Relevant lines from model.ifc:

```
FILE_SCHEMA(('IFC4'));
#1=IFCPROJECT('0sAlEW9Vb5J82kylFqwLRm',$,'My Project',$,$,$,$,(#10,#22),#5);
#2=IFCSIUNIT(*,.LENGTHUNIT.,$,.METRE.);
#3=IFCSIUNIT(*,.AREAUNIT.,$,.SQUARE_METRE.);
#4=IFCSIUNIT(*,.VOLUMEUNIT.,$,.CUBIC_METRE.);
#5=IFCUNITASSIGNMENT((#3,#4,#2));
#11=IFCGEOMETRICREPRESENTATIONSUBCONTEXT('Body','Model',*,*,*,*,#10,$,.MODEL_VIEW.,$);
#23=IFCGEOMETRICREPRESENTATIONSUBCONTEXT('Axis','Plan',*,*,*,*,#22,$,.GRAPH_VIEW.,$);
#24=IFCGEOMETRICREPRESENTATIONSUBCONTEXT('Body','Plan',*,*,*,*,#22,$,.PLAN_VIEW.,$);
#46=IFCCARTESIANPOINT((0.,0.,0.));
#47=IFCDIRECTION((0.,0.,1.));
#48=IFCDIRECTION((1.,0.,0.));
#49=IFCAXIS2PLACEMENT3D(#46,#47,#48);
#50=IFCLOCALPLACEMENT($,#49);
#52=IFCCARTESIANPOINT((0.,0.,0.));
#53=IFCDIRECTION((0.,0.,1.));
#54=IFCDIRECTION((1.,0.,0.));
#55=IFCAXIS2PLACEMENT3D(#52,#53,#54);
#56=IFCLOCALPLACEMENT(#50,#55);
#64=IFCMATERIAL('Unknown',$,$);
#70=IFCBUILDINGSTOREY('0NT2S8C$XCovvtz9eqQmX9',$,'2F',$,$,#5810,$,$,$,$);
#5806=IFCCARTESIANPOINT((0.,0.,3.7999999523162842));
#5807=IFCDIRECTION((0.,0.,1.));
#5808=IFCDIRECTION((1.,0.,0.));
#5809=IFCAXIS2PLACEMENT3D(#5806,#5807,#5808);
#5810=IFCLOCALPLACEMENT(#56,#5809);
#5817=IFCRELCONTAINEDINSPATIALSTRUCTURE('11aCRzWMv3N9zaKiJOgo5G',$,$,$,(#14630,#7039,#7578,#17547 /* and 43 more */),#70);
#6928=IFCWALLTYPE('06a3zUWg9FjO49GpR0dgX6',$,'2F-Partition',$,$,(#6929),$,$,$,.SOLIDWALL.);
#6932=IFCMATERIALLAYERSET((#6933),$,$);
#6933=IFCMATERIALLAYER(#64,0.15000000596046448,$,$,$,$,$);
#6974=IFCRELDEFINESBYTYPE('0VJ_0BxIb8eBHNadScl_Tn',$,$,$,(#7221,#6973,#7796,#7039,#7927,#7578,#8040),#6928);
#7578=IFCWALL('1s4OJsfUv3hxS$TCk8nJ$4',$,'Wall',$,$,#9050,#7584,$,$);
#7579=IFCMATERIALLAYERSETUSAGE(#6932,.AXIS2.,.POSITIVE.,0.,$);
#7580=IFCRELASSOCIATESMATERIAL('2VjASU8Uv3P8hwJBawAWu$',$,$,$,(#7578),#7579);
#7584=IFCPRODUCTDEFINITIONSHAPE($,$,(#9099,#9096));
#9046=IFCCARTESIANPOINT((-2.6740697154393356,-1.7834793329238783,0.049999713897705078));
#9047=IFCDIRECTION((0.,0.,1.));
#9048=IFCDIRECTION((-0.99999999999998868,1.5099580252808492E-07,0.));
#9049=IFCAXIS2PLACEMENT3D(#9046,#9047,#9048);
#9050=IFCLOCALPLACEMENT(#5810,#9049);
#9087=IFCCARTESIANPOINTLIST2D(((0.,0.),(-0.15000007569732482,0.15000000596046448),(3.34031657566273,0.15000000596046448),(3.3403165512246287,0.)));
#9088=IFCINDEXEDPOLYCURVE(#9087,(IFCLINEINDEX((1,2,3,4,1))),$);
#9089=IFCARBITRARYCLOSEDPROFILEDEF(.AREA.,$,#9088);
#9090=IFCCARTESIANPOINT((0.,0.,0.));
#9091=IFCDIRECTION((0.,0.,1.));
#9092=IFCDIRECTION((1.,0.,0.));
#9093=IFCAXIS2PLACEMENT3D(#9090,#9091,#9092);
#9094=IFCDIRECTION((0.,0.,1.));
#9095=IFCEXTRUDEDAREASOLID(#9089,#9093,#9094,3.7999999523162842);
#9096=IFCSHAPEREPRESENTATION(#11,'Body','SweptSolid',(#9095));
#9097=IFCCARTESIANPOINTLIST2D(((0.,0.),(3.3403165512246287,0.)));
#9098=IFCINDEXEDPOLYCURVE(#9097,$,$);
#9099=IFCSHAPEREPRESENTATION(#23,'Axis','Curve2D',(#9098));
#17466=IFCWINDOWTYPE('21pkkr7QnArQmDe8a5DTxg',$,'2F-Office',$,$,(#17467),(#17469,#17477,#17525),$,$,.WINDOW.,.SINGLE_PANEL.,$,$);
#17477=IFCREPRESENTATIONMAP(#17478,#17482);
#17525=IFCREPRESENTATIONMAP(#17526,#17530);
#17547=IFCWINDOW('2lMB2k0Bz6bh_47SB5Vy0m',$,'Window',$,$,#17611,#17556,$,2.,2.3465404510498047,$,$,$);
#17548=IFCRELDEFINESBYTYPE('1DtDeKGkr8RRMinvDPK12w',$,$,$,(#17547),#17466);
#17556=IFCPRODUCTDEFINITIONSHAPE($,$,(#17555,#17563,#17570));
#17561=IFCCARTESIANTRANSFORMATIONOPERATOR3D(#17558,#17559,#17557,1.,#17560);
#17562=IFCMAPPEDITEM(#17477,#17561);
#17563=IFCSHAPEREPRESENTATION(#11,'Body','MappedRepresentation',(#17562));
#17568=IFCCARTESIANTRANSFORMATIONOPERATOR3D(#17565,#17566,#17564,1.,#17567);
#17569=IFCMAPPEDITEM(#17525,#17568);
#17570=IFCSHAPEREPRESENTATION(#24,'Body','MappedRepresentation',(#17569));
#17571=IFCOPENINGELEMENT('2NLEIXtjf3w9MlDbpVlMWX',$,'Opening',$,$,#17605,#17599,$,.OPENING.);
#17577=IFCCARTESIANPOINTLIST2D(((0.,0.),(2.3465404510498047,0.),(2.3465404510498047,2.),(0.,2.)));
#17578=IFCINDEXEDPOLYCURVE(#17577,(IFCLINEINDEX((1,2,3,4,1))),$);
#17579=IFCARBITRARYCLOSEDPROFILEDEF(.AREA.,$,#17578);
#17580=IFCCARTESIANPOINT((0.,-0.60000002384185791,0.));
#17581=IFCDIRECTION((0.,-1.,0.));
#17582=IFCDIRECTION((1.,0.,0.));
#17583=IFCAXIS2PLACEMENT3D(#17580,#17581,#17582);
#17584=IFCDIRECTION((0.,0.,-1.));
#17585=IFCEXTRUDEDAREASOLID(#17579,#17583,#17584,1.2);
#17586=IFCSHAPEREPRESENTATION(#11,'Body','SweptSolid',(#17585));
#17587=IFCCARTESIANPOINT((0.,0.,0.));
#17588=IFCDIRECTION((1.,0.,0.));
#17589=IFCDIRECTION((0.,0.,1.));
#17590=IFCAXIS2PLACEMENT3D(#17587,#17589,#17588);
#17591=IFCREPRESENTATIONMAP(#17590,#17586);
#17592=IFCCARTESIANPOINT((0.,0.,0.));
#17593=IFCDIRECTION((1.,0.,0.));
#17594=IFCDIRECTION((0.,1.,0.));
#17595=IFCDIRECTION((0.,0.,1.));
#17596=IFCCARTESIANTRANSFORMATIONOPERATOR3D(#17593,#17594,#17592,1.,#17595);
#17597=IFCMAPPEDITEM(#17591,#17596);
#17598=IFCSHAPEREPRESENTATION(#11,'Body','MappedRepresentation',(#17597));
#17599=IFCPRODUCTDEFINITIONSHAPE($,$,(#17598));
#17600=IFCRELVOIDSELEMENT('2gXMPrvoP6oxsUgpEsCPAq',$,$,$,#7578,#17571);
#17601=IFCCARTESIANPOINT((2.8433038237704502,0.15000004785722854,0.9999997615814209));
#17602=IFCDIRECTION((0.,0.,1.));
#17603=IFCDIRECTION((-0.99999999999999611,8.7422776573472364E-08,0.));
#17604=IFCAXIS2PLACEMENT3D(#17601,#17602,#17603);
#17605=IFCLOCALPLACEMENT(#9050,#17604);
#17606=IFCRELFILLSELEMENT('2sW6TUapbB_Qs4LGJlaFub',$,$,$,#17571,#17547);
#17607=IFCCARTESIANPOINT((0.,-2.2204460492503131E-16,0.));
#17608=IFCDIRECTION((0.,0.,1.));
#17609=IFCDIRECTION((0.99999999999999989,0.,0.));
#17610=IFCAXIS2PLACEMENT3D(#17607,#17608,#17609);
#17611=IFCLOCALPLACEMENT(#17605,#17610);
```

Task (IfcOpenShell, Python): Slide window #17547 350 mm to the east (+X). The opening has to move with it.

```python
import ifcopenshell
import ifcopenshell.api.geometry
import ifcopenshell.util.placement
import ifcopenshell.util.unit

model = ifcopenshell.open("model.ifc")
unit_scale = ifcopenshell.util.unit.calculate_unit_scale(model)

window = model.by_id(17547)
opening = window.FillsVoids[0].RelatingOpeningElement
wall = opening.VoidsElements[0].RelatingBuildingElement

wall_matrix = ifcopenshell.util.placement.get_local_placement(wall.ObjectPlacement)
shift = wall_matrix[:3, 0] * -0.35 / unit_scale
before = ifcopenshell.util.placement.get_local_placement(window.ObjectPlacement)[:3, 3].copy()

# The window is placed relative to its opening, so it follows when the opening moves.
matrix = ifcopenshell.util.placement.get_local_placement(opening.ObjectPlacement)
matrix[:3, 3] += shift
ifcopenshell.api.geometry.edit_object_placement(
    model, product=opening, matrix=matrix, is_si=False, should_transform_children=True
)

after = ifcopenshell.util.placement.get_local_placement(window.ObjectPlacement)[:3, 3]
print("window moved by", (after - before).round(3) + 0.0)

model.write("model-out.ifc")
```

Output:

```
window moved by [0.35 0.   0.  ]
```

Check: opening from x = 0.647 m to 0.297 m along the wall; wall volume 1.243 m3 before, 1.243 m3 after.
